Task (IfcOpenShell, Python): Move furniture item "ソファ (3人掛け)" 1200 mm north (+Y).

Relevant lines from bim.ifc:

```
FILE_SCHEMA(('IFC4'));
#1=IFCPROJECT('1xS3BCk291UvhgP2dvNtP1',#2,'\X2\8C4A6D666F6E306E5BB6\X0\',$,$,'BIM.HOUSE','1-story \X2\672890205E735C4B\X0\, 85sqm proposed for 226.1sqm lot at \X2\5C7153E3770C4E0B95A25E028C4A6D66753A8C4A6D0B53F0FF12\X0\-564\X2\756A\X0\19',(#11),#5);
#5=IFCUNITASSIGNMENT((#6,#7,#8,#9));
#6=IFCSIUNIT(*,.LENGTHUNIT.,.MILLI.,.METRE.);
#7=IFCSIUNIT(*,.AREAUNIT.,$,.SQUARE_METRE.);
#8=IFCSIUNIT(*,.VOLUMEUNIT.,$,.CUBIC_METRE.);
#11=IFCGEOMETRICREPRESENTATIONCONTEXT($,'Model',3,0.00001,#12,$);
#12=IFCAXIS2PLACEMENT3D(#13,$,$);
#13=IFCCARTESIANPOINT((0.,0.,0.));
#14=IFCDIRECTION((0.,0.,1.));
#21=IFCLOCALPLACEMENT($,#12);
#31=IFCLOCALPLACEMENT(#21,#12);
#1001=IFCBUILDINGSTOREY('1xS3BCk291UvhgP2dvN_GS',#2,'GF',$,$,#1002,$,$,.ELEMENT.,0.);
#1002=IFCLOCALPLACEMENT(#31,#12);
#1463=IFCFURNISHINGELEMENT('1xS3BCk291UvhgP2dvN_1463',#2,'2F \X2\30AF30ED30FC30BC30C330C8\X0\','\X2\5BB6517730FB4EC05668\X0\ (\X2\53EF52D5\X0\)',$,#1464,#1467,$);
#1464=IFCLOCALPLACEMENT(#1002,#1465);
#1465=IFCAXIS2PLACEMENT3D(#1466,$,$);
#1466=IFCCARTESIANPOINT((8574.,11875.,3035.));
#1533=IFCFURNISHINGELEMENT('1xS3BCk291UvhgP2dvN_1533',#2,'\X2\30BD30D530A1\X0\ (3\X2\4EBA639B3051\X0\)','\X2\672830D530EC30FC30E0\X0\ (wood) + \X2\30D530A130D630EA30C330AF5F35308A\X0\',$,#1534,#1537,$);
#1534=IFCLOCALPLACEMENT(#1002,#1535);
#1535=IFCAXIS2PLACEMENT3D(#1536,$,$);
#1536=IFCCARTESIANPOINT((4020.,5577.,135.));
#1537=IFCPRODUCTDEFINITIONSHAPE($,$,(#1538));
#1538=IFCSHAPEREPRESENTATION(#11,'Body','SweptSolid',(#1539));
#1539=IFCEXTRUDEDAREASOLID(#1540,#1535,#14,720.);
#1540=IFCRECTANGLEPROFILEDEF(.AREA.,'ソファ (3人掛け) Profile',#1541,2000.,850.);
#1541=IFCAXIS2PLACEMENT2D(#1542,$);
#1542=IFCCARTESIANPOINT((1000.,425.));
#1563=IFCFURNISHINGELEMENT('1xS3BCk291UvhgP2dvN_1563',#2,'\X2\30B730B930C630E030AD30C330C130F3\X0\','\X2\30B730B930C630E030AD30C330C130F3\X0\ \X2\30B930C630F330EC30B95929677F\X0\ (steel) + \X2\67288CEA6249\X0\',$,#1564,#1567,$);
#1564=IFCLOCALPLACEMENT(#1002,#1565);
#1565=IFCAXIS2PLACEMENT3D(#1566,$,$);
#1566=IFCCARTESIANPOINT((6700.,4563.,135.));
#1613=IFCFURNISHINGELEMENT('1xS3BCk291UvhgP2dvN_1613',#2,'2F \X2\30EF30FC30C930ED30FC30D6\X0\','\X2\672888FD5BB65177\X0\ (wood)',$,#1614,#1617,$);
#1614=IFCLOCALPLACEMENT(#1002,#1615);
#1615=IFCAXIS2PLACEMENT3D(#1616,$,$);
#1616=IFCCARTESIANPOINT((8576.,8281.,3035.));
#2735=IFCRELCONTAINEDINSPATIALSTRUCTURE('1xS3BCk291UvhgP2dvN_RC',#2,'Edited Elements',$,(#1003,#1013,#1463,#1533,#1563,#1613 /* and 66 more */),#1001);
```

```python
import ifcopenshell
import ifcopenshell.api.geometry
import ifcopenshell.util.placement
import ifcopenshell.util.unit

model = ifcopenshell.open("bim.ifc")
unit_scale = ifcopenshell.util.unit.calculate_unit_scale(model)

item = model.by_id(1533)
matrix = ifcopenshell.util.placement.get_local_placement(item.ObjectPlacement)
matrix[1, 3] += 1.2 / unit_scale
ifcopenshell.api.geometry.edit_object_placement(model, product=item, matrix=matrix, is_si=False)

print(ifcopenshell.util.placement.get_local_placement(item.ObjectPlacement).round(3) + 0.0)

model.write("bim_updated.ifc")
```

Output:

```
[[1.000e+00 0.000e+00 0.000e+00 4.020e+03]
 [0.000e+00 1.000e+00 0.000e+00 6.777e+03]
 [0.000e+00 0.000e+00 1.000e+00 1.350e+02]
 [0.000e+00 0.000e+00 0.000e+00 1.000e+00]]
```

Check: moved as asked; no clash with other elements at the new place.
